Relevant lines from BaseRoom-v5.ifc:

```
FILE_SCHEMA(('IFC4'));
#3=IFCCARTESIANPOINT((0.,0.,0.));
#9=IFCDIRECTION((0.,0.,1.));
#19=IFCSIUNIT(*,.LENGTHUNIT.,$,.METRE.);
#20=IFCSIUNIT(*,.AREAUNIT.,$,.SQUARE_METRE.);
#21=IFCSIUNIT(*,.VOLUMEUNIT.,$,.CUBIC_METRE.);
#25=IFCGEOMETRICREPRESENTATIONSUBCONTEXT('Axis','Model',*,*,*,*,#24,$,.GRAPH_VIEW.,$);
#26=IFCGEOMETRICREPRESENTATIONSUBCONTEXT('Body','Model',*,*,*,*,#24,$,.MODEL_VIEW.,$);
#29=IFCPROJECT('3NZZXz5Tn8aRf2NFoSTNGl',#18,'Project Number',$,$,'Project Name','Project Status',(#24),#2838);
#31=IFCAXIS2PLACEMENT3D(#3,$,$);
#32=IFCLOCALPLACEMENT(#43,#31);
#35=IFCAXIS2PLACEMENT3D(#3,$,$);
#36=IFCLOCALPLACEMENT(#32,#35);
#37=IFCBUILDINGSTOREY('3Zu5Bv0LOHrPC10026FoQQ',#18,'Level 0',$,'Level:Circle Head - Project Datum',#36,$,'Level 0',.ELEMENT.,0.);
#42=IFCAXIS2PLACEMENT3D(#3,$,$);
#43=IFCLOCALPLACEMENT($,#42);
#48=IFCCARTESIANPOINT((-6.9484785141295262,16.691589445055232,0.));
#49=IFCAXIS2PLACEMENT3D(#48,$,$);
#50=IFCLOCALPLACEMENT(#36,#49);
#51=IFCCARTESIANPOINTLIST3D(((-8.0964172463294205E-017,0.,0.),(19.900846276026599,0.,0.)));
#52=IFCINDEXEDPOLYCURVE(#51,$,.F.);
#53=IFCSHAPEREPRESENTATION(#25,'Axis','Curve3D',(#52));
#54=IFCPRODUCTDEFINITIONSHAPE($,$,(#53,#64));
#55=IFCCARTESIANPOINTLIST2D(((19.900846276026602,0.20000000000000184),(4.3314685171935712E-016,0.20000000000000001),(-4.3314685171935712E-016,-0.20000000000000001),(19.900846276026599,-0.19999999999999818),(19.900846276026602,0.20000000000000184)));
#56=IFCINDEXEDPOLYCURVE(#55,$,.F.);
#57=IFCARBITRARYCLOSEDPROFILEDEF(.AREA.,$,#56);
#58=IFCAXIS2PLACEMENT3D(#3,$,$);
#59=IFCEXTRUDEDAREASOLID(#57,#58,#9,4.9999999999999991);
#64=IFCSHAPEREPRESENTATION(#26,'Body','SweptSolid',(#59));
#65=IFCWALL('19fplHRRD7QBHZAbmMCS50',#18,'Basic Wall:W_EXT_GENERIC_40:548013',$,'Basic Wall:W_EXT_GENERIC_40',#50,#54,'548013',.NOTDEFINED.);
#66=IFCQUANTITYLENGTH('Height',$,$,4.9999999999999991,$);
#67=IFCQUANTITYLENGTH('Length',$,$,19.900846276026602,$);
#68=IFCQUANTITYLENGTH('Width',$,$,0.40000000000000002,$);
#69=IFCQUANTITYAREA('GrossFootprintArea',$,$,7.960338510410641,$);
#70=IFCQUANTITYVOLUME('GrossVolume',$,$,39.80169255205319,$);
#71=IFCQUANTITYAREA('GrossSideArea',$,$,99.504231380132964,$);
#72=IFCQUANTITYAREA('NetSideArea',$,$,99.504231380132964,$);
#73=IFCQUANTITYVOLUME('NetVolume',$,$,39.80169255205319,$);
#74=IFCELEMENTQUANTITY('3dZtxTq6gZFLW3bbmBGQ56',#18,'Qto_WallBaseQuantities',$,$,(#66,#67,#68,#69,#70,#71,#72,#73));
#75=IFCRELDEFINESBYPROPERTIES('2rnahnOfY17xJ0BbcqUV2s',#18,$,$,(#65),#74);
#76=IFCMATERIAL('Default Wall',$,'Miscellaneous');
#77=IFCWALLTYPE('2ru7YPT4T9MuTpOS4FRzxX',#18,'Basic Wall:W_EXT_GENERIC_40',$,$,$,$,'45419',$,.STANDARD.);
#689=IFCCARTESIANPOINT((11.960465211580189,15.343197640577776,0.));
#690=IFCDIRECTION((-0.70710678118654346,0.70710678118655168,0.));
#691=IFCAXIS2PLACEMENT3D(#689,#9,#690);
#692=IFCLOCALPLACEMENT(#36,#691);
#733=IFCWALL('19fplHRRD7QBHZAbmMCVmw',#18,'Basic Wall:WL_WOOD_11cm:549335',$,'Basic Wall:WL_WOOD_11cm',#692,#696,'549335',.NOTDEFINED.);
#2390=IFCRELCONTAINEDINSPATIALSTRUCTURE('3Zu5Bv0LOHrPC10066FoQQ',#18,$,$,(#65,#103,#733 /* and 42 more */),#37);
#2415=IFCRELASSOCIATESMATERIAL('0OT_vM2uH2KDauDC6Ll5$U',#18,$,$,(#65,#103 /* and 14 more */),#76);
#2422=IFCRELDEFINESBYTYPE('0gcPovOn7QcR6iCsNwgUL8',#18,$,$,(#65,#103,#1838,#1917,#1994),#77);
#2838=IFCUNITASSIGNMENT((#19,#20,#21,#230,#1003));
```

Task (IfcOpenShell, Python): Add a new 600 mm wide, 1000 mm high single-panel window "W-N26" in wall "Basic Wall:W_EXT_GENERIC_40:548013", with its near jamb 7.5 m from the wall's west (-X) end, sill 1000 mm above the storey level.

```python
import numpy as np
import ifcopenshell
import ifcopenshell.api.feature
import ifcopenshell.api.geometry
import ifcopenshell.api.pset
import ifcopenshell.api.root
import ifcopenshell.api.spatial
import ifcopenshell.geom
import ifcopenshell.util.element
import ifcopenshell.util.placement
import ifcopenshell.util.representation
import ifcopenshell.util.shape
import ifcopenshell.util.unit

model = ifcopenshell.open("BaseRoom-v5.ifc")
unit_scale = ifcopenshell.util.unit.calculate_unit_scale(model)
area_scale = ifcopenshell.util.unit.calculate_unit_scale(model, "AREAUNIT")
volume_scale = ifcopenshell.util.unit.calculate_unit_scale(model, "VOLUMEUNIT")
settings = ifcopenshell.geom.settings()


def volume(element):
    """Net volume in cubic metres, openings subtracted."""
    shape = ifcopenshell.geom.create_shape(settings, element)
    return ifcopenshell.util.shape.get_volume(shape.geometry)


wall = model.by_guid("19fplHRRD7QBHZAbmMCS50")
storey = ifcopenshell.util.element.get_container(wall, ifc_class="IfcBuildingStorey")
context = ifcopenshell.util.representation.get_context(model, "Model", "Body", "MODEL_VIEW")
before = volume(wall)

width, height, from_end, sill = 0.6, 1, 7.5, 1  # metres

# The wall runs along its own X axis, and the end named is its -X end.
wall_shape = ifcopenshell.geom.create_shape(settings, wall)
x, y, z = ifcopenshell.util.shape.get_vertices(wall_shape.geometry).T
start = x.min() + from_end
face, thickness = float(y.min()), float(y.max() - y.min())
wall_matrix = ifcopenshell.util.placement.get_local_placement(wall.ObjectPlacement)
level = ifcopenshell.util.placement.get_local_placement(storey.ObjectPlacement)[2, 3]


def in_wall(x, y):
    """Placement at x, y metres in the wall's axes, at sill height."""
    matrix = wall_matrix.copy()
    matrix[:, 3] = wall_matrix @ np.array([x / unit_scale, y / unit_scale, 0.0, 1.0])
    matrix[2, 3] = level + sill / unit_scale
    return matrix


# Opening: a box that overshoots both wall faces by 50 mm.
opening = ifcopenshell.api.root.create_entity(model, ifc_class="IfcOpeningElement", predefined_type="OPENING")
box = ifcopenshell.api.geometry.add_wall_representation(
    model, context=context, length=width, height=height, thickness=thickness + 0.1
)
ifcopenshell.api.geometry.assign_representation(model, product=opening, representation=box)
ifcopenshell.api.geometry.edit_object_placement(model, product=opening, matrix=in_wall(start, face - 0.05), is_si=False)
ifcopenshell.api.feature.add_feature(model, feature=opening, element=wall)

window = ifcopenshell.api.root.create_entity(model, ifc_class="IfcWindow", name="W-N26", predefined_type="WINDOW")
window.OverallWidth, window.OverallHeight = width / unit_scale, height / unit_scale
window.PartitioningType = "SINGLE_PANEL"
body = ifcopenshell.api.geometry.add_window_representation(
    model,
    context=context,
    overall_width=window.OverallWidth,
    overall_height=window.OverallHeight,
    partition_type="SINGLE_PANEL",
)
ifcopenshell.api.geometry.assign_representation(model, product=window, representation=body)
ifcopenshell.api.spatial.assign_container(model, products=[window], relating_structure=storey)
ifcopenshell.api.feature.add_filling(model, opening=opening, element=window)

# Centre the window in the wall's thickness.
ifcopenshell.api.geometry.edit_object_placement(model, product=window, matrix=in_wall(start, face), is_si=False)
window_shape = ifcopenshell.geom.create_shape(settings, window)
depth = ifcopenshell.util.shape.get_vertices(window_shape.geometry)[:, 1]
offset = face + thickness / 2 - (depth.min() + depth.max()) / 2
ifcopenshell.api.geometry.edit_object_placement(model, product=window, matrix=in_wall(start, offset), is_si=False)

after = volume(wall)

# Update the wall's stored quantities.
qto = model.by_id(ifcopenshell.util.element.get_pset(wall, "Qto_WallBaseQuantities", should_inherit=False)["id"])
ifcopenshell.api.pset.edit_qto(model, qto=qto, properties={
    "NetSideArea": after / thickness / area_scale,
    "NetVolume": after / volume_scale,
})

print(f"wall volume {before:.3f} -> {after:.3f} m3")

model.write("BaseRoom-v5-out.ifc")
```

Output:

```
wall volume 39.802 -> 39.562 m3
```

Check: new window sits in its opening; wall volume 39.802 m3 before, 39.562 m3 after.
